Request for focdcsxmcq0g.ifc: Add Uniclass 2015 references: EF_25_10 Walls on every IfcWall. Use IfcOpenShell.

First a look at what the model holds.

```python
import ifcopenshell

model = ifcopenshell.open("focdcsxmcq0g.ifc")
print(model.schema)
print("classifications:", [c.Name for c in model.by_type("IfcClassification")])
for ifc_class in ("IfcDoor", "IfcRoof", "IfcStair", "IfcWall", "IfcWindow"):
    print(ifc_class, len(model.by_type(ifc_class)))
```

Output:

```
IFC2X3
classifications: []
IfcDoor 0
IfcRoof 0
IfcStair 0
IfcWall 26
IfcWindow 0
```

```python
import ifcopenshell
import ifcopenshell.api.classification

model = ifcopenshell.open("focdcsxmcq0g.ifc")

# IFC2X3 requires Source and Edition and has no link from the project to the system.
system = model.create_entity("IfcClassification", Source="NBS", Edition="2015", Name="Uniclass 2015")

codes = {
    "IfcWall": ("EF_25_10", "Walls"),
}
for ifc_class, (code, name) in codes.items():
    products = model.by_type(ifc_class)
    ifcopenshell.api.classification.add_reference(
        model, products=products, classification=system, identification=code, name=name
    )
    print(code, len(products))

model.write("focdcsxmcq0g_v2.ifc")
```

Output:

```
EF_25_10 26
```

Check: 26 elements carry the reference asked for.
